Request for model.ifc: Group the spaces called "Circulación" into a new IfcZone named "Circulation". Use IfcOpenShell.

First a look at what the model holds.

```python
import ifcopenshell

model = ifcopenshell.open("model.ifc")
print(model.schema)
seen = {}
for space in model.by_type("IfcSpace"):
    seen[space.LongName] = seen.get(space.LongName, 0) + 1
for name, count in sorted(seen.items(), key=str):
    print(count, "x", name)
print("zones:", [z.Name for z in model.by_type("IfcZone")][:20])
```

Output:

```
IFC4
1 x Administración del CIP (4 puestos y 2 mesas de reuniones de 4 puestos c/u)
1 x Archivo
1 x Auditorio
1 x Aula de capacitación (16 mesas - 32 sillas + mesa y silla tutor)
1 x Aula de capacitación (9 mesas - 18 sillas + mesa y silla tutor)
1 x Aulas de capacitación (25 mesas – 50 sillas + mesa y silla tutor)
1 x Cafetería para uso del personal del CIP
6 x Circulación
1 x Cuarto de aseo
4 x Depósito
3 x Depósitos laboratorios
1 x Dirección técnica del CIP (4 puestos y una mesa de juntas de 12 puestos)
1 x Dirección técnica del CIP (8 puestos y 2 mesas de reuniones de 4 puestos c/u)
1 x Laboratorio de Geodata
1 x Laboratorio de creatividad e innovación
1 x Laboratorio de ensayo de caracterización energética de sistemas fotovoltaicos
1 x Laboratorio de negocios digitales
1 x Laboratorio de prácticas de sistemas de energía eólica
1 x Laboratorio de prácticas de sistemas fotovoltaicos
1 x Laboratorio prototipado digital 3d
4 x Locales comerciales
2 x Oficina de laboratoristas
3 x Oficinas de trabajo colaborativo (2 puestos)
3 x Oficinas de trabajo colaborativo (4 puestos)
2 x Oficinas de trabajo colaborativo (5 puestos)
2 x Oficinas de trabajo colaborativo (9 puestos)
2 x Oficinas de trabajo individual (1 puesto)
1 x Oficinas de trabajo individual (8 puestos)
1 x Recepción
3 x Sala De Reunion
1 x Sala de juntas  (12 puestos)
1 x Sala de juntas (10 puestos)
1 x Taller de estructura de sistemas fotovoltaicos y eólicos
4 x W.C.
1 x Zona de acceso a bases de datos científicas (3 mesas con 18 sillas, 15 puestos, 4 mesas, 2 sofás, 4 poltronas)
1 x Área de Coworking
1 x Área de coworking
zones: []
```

```python
import ifcopenshell
import ifcopenshell.api.group
import ifcopenshell.api.root

model = ifcopenshell.open("model.ifc")

names = {"Circulación"}
spaces = [s for s in model.by_type("IfcSpace") if s.LongName in names]

zone = ifcopenshell.api.root.create_entity(model, ifc_class="IfcZone", name="Circulation")
ifcopenshell.api.group.assign_group(model, products=spaces, group=zone)
print(len(spaces), "spaces in", zone.Name)

model.write("model_v2.ifc")
```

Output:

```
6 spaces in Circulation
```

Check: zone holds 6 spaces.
